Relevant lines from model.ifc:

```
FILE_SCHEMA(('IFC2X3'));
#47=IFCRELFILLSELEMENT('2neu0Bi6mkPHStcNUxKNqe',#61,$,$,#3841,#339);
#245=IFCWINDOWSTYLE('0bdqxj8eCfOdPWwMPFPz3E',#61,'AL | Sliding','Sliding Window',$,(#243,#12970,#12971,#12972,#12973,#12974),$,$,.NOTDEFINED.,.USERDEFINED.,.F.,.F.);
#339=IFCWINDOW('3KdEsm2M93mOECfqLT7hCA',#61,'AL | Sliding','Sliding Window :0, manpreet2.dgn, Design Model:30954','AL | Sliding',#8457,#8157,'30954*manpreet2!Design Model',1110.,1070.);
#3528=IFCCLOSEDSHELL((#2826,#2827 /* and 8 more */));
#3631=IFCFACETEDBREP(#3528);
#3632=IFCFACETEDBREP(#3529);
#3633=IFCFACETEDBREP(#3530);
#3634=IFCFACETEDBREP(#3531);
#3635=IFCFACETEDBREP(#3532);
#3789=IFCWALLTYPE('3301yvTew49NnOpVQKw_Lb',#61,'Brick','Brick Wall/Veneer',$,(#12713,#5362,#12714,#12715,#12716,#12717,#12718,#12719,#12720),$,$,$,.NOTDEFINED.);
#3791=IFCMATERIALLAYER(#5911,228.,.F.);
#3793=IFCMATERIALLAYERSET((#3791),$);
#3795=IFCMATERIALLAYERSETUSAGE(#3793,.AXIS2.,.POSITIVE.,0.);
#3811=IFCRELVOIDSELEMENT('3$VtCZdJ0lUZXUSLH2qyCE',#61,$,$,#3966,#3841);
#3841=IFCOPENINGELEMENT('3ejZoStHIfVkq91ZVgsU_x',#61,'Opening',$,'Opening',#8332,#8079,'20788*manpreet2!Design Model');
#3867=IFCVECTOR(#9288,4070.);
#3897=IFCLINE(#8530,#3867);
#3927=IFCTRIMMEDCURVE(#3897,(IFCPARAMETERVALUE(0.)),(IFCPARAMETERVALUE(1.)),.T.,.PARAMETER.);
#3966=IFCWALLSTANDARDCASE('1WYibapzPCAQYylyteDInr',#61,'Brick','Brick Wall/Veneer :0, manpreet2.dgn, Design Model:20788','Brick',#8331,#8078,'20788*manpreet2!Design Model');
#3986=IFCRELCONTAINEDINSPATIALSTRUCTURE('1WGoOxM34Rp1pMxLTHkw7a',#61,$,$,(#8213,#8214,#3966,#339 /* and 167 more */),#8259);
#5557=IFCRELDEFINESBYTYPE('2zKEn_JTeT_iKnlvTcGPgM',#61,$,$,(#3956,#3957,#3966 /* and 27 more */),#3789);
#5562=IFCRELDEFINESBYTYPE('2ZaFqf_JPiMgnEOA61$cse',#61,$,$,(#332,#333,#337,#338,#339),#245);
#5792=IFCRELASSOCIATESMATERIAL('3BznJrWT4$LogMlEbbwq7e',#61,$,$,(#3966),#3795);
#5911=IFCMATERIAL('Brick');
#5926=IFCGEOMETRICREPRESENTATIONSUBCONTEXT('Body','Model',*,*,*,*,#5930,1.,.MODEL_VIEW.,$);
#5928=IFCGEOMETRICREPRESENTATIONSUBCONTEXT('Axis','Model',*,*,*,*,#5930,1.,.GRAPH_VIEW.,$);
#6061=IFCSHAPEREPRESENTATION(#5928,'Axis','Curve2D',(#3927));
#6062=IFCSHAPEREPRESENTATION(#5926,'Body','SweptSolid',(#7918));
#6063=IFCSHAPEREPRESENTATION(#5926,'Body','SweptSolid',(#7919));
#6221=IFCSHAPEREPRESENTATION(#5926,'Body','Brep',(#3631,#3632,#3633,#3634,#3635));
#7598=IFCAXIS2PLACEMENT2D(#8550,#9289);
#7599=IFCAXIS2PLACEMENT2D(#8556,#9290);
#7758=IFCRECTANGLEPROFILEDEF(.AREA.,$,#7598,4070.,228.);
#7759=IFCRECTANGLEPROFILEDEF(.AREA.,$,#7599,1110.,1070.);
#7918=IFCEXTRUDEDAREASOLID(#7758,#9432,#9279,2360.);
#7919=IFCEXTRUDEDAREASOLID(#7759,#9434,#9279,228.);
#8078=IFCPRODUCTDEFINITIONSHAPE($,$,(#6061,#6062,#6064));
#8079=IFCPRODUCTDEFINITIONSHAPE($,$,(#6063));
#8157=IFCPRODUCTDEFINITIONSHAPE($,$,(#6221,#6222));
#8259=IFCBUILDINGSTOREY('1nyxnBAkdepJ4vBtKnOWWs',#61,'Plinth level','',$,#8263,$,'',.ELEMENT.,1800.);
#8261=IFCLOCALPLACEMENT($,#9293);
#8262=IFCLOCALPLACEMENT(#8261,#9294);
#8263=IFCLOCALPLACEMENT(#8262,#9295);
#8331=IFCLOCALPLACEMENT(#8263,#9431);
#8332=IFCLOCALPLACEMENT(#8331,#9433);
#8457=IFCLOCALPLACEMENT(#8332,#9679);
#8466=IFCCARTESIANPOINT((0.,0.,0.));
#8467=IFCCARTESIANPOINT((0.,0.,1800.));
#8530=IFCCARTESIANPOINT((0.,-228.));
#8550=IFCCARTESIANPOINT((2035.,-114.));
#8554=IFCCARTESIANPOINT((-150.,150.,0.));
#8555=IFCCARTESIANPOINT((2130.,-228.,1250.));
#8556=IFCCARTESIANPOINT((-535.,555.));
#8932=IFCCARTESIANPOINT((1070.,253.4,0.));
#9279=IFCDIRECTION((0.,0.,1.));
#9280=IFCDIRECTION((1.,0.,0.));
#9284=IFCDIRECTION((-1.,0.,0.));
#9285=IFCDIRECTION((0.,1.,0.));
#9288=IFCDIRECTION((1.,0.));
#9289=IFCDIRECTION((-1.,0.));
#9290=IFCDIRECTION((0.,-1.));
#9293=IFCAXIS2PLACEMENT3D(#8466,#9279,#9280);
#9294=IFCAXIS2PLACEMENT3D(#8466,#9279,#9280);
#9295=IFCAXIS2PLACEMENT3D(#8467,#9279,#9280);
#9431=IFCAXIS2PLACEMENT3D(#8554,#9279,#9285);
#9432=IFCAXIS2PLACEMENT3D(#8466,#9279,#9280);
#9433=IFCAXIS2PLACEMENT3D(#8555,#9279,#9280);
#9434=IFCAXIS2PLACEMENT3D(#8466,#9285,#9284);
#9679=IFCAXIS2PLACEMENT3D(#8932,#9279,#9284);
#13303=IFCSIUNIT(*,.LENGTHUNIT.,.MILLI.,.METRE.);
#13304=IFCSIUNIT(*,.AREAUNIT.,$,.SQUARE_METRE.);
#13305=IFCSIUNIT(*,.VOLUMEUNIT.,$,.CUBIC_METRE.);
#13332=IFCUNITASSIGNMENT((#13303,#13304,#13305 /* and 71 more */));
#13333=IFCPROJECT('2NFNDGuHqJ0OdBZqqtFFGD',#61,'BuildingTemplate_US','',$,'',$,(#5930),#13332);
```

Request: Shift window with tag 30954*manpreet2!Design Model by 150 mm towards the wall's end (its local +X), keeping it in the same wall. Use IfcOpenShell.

```python
import ifcopenshell
import ifcopenshell.api.geometry
import ifcopenshell.util.placement

model = ifcopenshell.open("model.ifc")

window = model.by_guid("3KdEsm2M93mOECfqLT7hCA")
opening = window.FillsVoids[0].RelatingOpeningElement
wall = opening.VoidsElements[0].RelatingBuildingElement

wall_matrix = ifcopenshell.util.placement.get_local_placement(wall.ObjectPlacement)
shift = wall_matrix[:3, 0] * 150.0
before = ifcopenshell.util.placement.get_local_placement(window.ObjectPlacement)[:3, 3].copy()

# The window is placed relative to its opening, so it follows when the opening moves.
matrix = ifcopenshell.util.placement.get_local_placement(opening.ObjectPlacement)
matrix[:3, 3] += shift
ifcopenshell.api.geometry.edit_object_placement(
    model, product=opening, matrix=matrix, is_si=False, should_transform_children=True
)

after = ifcopenshell.util.placement.get_local_placement(window.ObjectPlacement)[:3, 3]
print("window moved by", (after - before).round(3) + 0.0)

model.write("model_updated.ifc")
```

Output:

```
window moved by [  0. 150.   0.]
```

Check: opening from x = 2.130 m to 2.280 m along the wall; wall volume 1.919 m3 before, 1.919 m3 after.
